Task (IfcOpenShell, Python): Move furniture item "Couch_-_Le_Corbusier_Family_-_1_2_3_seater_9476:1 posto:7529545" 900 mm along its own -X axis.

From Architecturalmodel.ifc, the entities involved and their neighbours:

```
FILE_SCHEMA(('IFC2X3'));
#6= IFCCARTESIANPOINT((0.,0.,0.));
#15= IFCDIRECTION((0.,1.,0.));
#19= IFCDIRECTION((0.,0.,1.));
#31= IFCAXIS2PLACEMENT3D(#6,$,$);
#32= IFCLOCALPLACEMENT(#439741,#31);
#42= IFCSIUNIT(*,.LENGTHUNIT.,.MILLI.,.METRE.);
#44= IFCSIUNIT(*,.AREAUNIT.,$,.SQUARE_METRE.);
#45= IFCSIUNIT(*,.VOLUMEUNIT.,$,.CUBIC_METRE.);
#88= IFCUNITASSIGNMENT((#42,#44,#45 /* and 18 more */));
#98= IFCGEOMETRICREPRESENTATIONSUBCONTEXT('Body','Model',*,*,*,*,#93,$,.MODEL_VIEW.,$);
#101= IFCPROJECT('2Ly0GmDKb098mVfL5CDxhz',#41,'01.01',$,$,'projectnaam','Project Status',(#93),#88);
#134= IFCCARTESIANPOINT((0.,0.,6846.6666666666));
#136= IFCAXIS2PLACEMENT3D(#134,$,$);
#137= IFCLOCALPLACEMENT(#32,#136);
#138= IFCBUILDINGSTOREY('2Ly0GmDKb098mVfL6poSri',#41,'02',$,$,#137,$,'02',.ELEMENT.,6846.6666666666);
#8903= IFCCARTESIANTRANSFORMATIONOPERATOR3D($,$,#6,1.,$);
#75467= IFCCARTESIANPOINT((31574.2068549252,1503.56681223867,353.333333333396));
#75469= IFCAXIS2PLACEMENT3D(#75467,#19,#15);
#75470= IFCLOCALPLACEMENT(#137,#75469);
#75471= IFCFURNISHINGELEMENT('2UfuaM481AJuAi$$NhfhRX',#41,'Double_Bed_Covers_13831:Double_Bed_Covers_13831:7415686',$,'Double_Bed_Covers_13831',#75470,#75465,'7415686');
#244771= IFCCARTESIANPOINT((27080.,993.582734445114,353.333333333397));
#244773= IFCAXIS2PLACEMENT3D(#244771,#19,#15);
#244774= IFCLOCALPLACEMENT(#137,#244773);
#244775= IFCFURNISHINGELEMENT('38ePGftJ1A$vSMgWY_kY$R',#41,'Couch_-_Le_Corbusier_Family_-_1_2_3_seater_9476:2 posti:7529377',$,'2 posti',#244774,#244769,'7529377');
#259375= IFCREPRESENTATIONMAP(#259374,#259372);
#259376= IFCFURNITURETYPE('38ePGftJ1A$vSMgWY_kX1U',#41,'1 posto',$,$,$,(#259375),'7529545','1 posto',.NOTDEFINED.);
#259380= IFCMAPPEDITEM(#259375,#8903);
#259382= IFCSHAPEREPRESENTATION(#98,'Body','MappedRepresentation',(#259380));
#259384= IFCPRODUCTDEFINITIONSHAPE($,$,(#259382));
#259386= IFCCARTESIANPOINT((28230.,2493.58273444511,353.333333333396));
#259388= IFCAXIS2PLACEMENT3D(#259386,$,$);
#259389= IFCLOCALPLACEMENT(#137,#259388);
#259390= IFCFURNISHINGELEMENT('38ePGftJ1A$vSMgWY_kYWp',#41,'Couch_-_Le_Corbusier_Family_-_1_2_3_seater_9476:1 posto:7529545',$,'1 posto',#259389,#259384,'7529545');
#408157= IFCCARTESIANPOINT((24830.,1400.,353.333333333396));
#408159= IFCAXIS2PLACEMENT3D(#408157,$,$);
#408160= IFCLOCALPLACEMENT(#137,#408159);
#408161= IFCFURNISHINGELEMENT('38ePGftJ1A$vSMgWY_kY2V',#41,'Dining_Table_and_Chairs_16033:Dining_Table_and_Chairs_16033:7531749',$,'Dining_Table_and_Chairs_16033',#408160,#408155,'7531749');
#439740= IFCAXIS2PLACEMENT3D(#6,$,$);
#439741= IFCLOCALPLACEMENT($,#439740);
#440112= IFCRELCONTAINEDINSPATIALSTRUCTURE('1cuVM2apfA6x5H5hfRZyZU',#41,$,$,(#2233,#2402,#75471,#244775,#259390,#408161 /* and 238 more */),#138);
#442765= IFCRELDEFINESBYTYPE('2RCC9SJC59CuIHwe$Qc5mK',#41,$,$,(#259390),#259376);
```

```python
import ifcopenshell
import ifcopenshell.api.geometry
import ifcopenshell.util.placement

model = ifcopenshell.open("Architecturalmodel.ifc")

item = model.by_id(259390)
matrix = ifcopenshell.util.placement.get_local_placement(item.ObjectPlacement)
matrix[:3, 3] -= matrix[:3, 0] * 900.0
ifcopenshell.api.geometry.edit_object_placement(model, product=item, matrix=matrix, is_si=False)

print(ifcopenshell.util.placement.get_local_placement(item.ObjectPlacement).round(3) + 0.0)

model.write("Architecturalmodel-out.ifc")
```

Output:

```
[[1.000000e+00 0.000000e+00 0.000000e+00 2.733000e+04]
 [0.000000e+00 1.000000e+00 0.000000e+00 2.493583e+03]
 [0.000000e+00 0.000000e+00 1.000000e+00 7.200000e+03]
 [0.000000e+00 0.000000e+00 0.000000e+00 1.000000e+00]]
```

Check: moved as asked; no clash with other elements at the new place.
